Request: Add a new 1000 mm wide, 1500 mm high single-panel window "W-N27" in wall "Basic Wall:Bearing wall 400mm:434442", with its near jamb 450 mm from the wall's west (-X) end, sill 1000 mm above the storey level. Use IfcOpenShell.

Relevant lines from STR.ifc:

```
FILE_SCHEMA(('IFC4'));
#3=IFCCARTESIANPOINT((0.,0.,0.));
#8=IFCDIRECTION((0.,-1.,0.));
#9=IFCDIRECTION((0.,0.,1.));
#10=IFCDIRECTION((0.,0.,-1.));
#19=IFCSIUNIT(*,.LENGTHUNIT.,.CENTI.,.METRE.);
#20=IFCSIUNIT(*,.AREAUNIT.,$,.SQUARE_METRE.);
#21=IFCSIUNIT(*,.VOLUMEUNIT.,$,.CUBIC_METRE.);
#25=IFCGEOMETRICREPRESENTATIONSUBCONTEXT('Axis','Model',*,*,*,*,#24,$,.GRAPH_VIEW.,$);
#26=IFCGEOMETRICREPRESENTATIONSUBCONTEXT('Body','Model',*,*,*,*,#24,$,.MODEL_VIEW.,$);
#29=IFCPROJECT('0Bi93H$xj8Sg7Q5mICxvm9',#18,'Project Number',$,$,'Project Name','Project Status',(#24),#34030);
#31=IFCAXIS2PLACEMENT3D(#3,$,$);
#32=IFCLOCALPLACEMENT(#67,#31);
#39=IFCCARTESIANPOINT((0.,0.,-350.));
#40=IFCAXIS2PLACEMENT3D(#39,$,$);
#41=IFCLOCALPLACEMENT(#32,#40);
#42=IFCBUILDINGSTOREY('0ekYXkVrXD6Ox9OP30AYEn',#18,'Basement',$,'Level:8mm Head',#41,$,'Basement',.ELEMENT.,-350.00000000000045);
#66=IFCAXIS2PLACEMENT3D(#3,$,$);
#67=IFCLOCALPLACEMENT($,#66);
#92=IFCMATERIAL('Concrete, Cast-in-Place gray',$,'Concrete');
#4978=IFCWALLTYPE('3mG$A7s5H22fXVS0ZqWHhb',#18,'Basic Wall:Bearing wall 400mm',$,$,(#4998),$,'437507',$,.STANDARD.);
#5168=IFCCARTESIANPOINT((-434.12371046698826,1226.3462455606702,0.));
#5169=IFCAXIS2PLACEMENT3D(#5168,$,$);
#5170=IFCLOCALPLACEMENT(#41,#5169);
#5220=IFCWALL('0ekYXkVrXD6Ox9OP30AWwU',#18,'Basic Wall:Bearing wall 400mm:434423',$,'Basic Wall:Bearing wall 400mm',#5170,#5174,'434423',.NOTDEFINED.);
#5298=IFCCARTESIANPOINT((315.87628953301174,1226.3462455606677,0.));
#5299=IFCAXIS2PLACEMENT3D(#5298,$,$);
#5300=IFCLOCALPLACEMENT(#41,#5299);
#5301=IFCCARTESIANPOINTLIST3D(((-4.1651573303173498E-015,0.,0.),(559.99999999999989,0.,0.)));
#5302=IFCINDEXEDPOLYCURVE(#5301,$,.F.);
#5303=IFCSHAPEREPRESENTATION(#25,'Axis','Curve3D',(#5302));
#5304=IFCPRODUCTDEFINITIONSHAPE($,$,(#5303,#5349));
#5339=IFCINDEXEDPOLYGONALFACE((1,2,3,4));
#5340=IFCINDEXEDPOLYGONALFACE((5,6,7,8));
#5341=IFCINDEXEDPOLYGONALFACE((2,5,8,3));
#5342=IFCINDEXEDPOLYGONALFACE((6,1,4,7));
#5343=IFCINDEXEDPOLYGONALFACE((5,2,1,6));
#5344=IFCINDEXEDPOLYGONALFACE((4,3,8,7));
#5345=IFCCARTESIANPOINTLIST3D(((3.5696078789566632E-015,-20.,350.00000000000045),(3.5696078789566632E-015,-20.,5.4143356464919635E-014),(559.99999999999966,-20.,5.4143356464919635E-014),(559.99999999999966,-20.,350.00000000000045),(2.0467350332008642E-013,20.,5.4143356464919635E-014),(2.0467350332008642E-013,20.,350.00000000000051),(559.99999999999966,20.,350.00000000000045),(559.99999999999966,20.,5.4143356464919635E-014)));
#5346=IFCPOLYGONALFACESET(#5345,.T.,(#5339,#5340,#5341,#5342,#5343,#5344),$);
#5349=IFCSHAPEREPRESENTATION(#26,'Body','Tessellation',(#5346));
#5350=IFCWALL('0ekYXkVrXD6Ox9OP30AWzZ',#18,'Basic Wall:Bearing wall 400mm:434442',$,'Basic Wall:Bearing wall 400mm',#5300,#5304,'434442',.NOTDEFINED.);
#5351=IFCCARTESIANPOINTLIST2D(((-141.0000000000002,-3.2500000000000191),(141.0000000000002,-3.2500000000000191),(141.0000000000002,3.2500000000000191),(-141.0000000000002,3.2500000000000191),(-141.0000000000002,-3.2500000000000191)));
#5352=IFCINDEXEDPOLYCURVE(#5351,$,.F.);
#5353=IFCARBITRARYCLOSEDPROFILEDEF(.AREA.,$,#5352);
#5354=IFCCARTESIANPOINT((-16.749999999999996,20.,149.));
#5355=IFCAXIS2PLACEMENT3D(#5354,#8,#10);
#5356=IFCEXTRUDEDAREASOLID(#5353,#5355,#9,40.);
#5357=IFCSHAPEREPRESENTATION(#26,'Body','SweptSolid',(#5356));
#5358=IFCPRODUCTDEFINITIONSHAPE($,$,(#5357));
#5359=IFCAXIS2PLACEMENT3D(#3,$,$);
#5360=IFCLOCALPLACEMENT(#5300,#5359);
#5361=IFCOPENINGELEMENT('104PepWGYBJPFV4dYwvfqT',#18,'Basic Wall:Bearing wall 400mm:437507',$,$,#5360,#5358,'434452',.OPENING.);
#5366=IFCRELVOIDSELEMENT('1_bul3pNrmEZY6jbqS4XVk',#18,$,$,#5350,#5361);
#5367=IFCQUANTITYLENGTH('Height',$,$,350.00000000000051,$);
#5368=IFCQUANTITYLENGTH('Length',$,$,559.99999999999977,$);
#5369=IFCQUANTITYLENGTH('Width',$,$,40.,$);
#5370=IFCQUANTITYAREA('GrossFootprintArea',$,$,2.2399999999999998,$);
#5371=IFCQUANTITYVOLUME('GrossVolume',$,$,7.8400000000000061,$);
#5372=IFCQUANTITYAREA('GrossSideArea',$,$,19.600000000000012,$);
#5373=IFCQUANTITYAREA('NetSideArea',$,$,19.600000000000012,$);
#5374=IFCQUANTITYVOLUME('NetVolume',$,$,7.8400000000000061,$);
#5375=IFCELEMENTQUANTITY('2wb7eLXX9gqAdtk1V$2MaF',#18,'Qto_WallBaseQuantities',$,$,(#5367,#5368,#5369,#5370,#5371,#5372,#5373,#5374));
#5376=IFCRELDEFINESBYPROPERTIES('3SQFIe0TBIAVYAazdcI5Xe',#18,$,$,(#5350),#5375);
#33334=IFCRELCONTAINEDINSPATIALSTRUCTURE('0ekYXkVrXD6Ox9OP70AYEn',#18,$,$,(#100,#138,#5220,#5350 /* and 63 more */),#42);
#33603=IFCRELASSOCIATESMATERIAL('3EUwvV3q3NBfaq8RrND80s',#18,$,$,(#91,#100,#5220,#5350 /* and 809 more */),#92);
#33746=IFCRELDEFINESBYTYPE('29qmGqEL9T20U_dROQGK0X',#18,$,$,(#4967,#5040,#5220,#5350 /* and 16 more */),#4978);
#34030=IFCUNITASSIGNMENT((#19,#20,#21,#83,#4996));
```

```python
import numpy as np
import ifcopenshell
import ifcopenshell.api.feature
import ifcopenshell.api.geometry
import ifcopenshell.api.pset
import ifcopenshell.api.root
import ifcopenshell.api.spatial
import ifcopenshell.geom
import ifcopenshell.util.element
import ifcopenshell.util.placement
import ifcopenshell.util.representation
import ifcopenshell.util.shape
import ifcopenshell.util.unit

model = ifcopenshell.open("STR.ifc")
unit_scale = ifcopenshell.util.unit.calculate_unit_scale(model)
area_scale = ifcopenshell.util.unit.calculate_unit_scale(model, "AREAUNIT")
volume_scale = ifcopenshell.util.unit.calculate_unit_scale(model, "VOLUMEUNIT")
settings = ifcopenshell.geom.settings()


def volume(element):
    """Net volume in cubic metres, openings subtracted."""
    shape = ifcopenshell.geom.create_shape(settings, element)
    return ifcopenshell.util.shape.get_volume(shape.geometry)


wall = model.by_guid("0ekYXkVrXD6Ox9OP30AWzZ")
storey = ifcopenshell.util.element.get_container(wall, ifc_class="IfcBuildingStorey")
context = ifcopenshell.util.representation.get_context(model, "Model", "Body", "MODEL_VIEW")
before = volume(wall)

width, height, from_end, sill = 1, 1.5, 0.45, 1  # metres

# The wall runs along its own X axis, and the end named is its -X end.
wall_shape = ifcopenshell.geom.create_shape(settings, wall)
x, y, z = ifcopenshell.util.shape.get_vertices(wall_shape.geometry).T
start = x.min() + from_end
face, thickness = float(y.min()), float(y.max() - y.min())
wall_matrix = ifcopenshell.util.placement.get_local_placement(wall.ObjectPlacement)
level = ifcopenshell.util.placement.get_local_placement(storey.ObjectPlacement)[2, 3]


def in_wall(x, y):
    """Placement at x, y metres in the wall's axes, at sill height."""
    matrix = wall_matrix.copy()
    matrix[:, 3] = wall_matrix @ np.array([x / unit_scale, y / unit_scale, 0.0, 1.0])
    matrix[2, 3] = level + sill / unit_scale
    return matrix


# Opening: a box that overshoots both wall faces by 50 mm.
opening = ifcopenshell.api.root.create_entity(model, ifc_class="IfcOpeningElement", predefined_type="OPENING")
box = ifcopenshell.api.geometry.add_wall_representation(
    model, context=context, length=width, height=height, thickness=thickness + 0.1
)
ifcopenshell.api.geometry.assign_representation(model, product=opening, representation=box)
ifcopenshell.api.geometry.edit_object_placement(model, product=opening, matrix=in_wall(start, face - 0.05), is_si=False)
ifcopenshell.api.feature.add_feature(model, feature=opening, element=wall)

window = ifcopenshell.api.root.create_entity(model, ifc_class="IfcWindow", name="W-N27", predefined_type="WINDOW")
window.OverallWidth, window.OverallHeight = width / unit_scale, height / unit_scale
window.PartitioningType = "SINGLE_PANEL"
body = ifcopenshell.api.geometry.add_window_representation(
    model,
    context=context,
    overall_width=window.OverallWidth,
    overall_height=window.OverallHeight,
    partition_type="SINGLE_PANEL",
)
ifcopenshell.api.geometry.assign_representation(model, product=window, representation=body)
ifcopenshell.api.spatial.assign_container(model, products=[window], relating_structure=storey)
ifcopenshell.api.feature.add_filling(model, opening=opening, element=window)

# Centre the window in the wall's thickness.
ifcopenshell.api.geometry.edit_object_placement(model, product=window, matrix=in_wall(start, face), is_si=False)
window_shape = ifcopenshell.geom.create_shape(settings, window)
depth = ifcopenshell.util.shape.get_vertices(window_shape.geometry)[:, 1]
offset = face + thickness / 2 - (depth.min() + depth.max()) / 2
ifcopenshell.api.geometry.edit_object_placement(model, product=window, matrix=in_wall(start, offset), is_si=False)

after = volume(wall)

# Update the wall's stored quantities.
qto = model.by_id(ifcopenshell.util.element.get_pset(wall, "Qto_WallBaseQuantities", should_inherit=False)["id"])
ifcopenshell.api.pset.edit_qto(model, qto=qto, properties={
    "NetSideArea": after / thickness / area_scale,
    "NetVolume": after / volume_scale,
})

print(f"wall volume {before:.3f} -> {after:.3f} m3")

model.write("STR_updated.ifc")
```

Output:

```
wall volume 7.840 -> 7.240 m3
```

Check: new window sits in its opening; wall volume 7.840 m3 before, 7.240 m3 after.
